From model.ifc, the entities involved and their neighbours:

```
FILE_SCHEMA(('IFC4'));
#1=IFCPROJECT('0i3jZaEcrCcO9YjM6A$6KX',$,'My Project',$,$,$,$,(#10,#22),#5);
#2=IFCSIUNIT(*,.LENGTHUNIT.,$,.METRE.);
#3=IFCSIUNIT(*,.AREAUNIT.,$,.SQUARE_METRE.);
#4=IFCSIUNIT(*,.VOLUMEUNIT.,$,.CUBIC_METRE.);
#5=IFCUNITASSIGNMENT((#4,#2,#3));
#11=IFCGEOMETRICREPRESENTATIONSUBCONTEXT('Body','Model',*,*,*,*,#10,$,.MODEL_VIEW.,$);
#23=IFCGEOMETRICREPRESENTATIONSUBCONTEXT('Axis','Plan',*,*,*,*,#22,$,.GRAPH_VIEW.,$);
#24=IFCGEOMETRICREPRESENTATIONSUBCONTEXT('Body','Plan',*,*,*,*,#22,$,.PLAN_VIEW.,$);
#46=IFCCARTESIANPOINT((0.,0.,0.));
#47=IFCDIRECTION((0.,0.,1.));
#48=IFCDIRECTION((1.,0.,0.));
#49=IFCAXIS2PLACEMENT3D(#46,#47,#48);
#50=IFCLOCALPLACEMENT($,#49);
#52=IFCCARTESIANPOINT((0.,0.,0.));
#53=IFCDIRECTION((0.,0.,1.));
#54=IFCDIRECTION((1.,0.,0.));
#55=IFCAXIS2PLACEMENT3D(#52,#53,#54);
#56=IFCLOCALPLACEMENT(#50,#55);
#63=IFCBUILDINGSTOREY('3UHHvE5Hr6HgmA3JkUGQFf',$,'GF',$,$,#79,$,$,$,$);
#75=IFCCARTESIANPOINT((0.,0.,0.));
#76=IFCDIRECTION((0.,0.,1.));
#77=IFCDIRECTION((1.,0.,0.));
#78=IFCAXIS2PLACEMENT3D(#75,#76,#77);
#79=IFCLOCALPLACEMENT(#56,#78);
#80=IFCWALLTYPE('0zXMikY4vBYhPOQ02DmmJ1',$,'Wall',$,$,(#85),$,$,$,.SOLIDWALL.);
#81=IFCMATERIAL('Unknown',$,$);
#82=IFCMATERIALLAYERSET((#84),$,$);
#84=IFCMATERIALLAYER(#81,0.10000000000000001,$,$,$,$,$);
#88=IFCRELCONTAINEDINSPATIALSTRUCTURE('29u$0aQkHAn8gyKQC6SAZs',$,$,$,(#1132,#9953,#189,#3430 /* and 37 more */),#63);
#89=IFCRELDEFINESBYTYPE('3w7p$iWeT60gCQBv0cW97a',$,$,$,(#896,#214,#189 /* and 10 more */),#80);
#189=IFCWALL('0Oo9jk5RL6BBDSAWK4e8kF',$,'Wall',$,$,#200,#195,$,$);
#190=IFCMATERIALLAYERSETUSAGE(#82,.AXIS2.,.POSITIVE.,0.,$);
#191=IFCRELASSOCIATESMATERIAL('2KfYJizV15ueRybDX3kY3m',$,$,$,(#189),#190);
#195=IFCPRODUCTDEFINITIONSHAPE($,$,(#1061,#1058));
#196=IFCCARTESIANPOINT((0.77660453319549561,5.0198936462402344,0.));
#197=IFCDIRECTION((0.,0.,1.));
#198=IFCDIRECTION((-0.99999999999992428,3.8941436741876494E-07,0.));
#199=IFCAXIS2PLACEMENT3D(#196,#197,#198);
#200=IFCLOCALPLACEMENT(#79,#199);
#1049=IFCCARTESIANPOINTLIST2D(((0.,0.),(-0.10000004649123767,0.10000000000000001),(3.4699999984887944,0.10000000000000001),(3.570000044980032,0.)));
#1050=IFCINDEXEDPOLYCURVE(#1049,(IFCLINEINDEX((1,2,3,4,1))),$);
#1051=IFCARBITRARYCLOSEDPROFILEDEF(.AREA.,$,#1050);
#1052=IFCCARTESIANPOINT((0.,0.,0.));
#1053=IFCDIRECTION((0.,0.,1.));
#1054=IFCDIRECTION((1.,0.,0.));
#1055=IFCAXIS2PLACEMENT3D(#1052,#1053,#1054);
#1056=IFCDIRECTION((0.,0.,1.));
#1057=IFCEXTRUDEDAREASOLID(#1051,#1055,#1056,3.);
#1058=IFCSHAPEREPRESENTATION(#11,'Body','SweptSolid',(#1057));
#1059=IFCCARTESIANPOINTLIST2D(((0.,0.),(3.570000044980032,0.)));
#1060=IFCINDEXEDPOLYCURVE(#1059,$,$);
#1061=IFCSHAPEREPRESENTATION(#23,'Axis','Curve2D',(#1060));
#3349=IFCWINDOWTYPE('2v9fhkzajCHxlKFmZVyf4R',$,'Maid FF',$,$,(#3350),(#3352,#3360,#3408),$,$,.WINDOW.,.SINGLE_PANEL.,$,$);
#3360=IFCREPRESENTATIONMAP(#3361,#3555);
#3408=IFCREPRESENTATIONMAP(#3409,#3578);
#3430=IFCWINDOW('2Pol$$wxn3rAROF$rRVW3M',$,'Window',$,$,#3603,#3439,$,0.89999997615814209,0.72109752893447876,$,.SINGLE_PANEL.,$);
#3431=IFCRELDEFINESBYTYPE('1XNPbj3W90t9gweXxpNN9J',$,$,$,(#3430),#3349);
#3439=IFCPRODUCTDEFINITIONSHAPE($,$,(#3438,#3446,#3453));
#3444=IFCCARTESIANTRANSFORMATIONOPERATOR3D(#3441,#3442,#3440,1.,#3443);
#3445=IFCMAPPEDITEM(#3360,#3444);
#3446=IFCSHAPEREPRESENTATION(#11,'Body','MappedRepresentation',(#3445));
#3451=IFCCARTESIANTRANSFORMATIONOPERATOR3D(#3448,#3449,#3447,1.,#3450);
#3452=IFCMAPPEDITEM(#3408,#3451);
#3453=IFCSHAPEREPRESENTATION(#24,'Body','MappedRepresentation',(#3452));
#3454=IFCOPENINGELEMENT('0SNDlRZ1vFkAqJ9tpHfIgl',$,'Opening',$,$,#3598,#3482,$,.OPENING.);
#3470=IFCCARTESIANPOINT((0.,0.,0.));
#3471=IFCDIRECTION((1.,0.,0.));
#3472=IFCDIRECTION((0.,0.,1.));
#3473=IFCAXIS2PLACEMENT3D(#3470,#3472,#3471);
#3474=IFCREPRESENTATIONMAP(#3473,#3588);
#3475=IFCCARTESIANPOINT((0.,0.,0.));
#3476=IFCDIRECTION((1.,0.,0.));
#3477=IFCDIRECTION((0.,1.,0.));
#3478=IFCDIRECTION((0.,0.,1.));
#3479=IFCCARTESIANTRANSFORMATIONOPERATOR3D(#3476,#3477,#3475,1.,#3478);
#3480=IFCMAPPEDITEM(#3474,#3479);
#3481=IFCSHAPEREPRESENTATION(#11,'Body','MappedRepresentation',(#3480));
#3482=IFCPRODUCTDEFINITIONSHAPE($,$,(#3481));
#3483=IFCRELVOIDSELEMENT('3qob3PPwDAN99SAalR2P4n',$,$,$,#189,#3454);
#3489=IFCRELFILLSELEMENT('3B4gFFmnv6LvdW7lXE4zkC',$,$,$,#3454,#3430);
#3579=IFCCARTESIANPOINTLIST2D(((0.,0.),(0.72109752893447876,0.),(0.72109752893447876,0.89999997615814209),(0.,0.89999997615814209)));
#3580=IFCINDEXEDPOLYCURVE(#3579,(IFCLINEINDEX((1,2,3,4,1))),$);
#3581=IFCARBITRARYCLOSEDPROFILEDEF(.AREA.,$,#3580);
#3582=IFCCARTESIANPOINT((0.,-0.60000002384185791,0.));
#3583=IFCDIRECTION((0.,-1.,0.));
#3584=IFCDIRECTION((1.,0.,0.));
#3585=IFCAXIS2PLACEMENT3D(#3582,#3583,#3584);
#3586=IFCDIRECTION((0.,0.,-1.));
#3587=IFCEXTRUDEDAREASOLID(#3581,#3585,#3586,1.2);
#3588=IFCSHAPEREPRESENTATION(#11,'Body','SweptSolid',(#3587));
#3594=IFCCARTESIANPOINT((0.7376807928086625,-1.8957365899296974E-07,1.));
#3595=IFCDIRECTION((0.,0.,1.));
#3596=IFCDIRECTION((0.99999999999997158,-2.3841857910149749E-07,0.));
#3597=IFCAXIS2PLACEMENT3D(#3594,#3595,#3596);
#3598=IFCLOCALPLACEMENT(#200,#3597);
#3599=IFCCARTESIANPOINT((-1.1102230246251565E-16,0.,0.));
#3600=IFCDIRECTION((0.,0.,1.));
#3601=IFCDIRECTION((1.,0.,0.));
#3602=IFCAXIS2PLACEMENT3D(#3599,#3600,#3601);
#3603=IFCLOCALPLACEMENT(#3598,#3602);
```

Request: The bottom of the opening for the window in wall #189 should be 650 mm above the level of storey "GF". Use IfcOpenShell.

```python
import numpy as np
import ifcopenshell
import ifcopenshell.api.geometry
import ifcopenshell.geom
import ifcopenshell.util.element
import ifcopenshell.util.placement
import ifcopenshell.util.shape
import ifcopenshell.util.unit

model = ifcopenshell.open("model.ifc")
unit_scale = ifcopenshell.util.unit.calculate_unit_scale(model)

window = model.by_guid("2Pol$$wxn3rAROF$rRVW3M")
opening = window.FillsVoids[0].RelatingOpeningElement
storey = ifcopenshell.util.element.get_container(window, ifc_class="IfcBuildingStorey")
level = ifcopenshell.util.placement.get_local_placement(storey.ObjectPlacement)[2, 3]

# The opening's origin need not be at the sill, so measure its lowest point.
shape = ifcopenshell.geom.create_shape(ifcopenshell.geom.settings(), opening)
bottom = ifcopenshell.util.shape.get_shape_bottom_elevation(shape, shape.geometry) / unit_scale
dz = level + 0.65 / unit_scale - bottom

shift = np.array([0.0, 0.0, dz])
# The window is placed relative to its opening, so it follows when the opening moves.
matrix = ifcopenshell.util.placement.get_local_placement(opening.ObjectPlacement)
matrix[:3, 3] += shift
ifcopenshell.api.geometry.edit_object_placement(
    model, product=opening, matrix=matrix, is_si=False, should_transform_children=True
)

print(f"moved by {dz * unit_scale:+.3f} m")

model.write("model_v2.ifc")
```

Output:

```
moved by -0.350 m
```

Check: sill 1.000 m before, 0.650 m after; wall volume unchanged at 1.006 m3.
